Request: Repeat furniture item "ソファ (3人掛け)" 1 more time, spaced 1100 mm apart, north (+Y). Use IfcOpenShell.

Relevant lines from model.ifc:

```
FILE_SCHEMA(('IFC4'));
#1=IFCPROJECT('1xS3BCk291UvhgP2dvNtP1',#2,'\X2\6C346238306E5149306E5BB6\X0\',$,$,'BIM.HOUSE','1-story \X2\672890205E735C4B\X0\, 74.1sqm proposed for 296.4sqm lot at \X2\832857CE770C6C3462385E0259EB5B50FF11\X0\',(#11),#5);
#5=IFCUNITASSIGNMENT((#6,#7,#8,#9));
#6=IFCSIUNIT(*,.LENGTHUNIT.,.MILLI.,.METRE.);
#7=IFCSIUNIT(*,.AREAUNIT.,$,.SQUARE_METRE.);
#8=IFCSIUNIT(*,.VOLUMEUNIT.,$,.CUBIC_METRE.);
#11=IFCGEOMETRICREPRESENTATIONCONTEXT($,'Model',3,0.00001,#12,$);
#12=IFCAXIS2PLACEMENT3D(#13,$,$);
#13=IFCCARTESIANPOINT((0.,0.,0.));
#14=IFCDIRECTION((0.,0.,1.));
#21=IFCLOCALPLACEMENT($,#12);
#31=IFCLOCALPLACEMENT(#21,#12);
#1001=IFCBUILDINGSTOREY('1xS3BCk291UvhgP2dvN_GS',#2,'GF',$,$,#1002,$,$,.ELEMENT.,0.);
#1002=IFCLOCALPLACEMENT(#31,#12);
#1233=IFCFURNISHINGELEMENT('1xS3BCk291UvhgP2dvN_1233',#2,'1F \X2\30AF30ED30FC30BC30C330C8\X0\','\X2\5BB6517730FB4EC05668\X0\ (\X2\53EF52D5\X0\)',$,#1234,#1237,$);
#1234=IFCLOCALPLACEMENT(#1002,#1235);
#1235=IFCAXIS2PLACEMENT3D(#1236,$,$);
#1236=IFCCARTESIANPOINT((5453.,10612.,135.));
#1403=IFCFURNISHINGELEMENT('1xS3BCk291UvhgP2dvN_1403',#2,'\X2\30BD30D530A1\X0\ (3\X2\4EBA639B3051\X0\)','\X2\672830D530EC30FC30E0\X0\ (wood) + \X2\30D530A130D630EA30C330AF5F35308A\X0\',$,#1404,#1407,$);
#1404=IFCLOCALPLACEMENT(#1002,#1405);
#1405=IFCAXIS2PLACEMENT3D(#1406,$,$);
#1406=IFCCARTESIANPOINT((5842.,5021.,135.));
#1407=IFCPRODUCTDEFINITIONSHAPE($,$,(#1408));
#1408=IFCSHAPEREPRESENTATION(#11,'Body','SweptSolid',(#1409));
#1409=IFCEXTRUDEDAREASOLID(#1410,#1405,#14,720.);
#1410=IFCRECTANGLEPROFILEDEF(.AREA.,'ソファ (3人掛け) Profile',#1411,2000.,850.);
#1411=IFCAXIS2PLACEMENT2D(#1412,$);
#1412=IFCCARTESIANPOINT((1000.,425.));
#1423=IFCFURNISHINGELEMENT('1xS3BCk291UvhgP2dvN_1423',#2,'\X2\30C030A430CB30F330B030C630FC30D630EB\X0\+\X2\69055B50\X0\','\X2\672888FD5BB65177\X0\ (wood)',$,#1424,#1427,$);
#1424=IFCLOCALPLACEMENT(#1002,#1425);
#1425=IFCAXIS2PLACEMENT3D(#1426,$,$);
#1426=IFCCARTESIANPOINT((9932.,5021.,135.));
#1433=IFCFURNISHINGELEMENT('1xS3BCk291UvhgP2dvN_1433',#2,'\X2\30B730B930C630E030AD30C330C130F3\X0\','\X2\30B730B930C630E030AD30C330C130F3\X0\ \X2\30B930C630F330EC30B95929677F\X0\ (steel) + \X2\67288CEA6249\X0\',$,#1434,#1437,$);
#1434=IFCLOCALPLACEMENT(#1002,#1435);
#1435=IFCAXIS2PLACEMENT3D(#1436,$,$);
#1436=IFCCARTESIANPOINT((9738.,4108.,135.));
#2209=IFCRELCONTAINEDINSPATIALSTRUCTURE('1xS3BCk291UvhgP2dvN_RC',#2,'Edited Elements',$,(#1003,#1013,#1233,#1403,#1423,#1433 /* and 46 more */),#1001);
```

```python
import numpy as np
import ifcopenshell
import ifcopenshell.api.geometry
import ifcopenshell.api.root
import ifcopenshell.util.element
import ifcopenshell.util.placement

model = ifcopenshell.open("model.ifc")


def reuse_history(source, copy):
    """copy_class also copies each property set's owner history, people and application; keep the originals."""
    for rel in copy.IsDefinedBy:
        if rel.is_a("IfcRelDefinesByProperties") and (history := rel.RelatingPropertyDefinition.OwnerHistory):
            rel.RelatingPropertyDefinition.OwnerHistory = source.OwnerHistory
            ifcopenshell.util.element.remove_deep2(model, history)


source = model.by_guid("1xS3BCk291UvhgP2dvN_1403")
base = ifcopenshell.util.placement.get_local_placement(source.ObjectPlacement)
step = np.array([0.0, 1.0, 0.0]) * 1100.0

for i in range(1, 2):
    copy = ifcopenshell.api.root.copy_class(model, product=source)
    copy.Representation = ifcopenshell.util.element.copy_deep(
        model, source.Representation, exclude=["IfcGeometricRepresentationContext", "IfcRepresentationMap"]
    )
    reuse_history(source, copy)
    matrix = base.copy()
    matrix[:3, 3] += i * step
    print("added at", matrix[:3, 3].round(3) + 0.0)
    ifcopenshell.api.geometry.edit_object_placement(model, product=copy, matrix=matrix, is_si=False)

model.write("model_rev.ifc")
```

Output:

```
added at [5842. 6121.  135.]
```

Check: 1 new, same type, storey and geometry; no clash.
